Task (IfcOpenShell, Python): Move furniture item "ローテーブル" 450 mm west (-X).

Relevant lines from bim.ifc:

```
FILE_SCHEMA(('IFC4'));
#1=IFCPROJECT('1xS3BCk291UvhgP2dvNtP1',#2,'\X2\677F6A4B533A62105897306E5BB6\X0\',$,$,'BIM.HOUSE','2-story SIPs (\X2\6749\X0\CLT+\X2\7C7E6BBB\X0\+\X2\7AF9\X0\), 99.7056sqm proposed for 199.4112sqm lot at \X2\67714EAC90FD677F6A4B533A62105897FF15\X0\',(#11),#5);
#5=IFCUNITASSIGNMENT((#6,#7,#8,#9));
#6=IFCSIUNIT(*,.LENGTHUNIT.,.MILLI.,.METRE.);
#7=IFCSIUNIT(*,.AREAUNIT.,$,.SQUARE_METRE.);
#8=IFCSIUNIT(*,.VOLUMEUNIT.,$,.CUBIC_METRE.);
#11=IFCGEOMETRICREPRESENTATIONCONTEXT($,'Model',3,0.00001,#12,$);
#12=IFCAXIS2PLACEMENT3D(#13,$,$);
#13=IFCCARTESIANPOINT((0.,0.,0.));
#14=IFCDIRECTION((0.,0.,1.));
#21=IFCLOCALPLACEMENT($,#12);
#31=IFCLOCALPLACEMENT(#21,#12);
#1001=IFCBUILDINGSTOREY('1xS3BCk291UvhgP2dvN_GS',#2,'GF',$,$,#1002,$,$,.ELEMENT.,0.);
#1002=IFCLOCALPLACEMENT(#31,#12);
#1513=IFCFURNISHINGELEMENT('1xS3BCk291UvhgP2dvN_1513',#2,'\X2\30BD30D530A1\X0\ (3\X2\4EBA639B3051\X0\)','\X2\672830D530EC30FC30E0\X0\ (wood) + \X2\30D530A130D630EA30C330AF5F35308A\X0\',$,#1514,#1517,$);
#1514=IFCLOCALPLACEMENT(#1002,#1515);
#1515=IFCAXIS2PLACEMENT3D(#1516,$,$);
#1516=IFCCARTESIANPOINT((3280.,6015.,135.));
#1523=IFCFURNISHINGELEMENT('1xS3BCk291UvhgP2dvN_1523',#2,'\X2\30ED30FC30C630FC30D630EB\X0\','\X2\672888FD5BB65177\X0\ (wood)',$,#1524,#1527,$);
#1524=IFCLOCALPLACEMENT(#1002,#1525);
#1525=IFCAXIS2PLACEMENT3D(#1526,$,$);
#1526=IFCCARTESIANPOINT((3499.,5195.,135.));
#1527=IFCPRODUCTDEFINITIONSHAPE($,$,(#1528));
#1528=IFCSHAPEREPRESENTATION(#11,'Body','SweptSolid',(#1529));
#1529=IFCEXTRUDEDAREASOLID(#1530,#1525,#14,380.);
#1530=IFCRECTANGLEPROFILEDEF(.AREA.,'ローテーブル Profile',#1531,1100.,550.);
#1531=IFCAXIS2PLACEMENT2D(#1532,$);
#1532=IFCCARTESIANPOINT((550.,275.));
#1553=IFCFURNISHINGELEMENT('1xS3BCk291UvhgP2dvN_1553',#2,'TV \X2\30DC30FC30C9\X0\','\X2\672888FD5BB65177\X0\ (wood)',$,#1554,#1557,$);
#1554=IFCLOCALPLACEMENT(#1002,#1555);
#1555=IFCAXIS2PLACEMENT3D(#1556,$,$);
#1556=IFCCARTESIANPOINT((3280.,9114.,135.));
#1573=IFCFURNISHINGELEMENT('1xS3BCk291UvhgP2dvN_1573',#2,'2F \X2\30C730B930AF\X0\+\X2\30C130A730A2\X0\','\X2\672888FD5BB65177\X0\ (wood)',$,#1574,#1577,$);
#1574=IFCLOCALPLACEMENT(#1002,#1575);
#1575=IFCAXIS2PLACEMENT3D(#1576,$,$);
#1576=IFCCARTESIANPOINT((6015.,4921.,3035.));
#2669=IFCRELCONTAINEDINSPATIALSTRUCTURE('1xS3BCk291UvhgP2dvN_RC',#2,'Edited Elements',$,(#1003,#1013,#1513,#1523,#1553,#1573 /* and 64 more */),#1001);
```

```python
import ifcopenshell
import ifcopenshell.api.geometry
import ifcopenshell.util.placement
import ifcopenshell.util.unit

model = ifcopenshell.open("bim.ifc")
unit_scale = ifcopenshell.util.unit.calculate_unit_scale(model)

item = model.by_id(1523)
matrix = ifcopenshell.util.placement.get_local_placement(item.ObjectPlacement)
matrix[0, 3] -= 0.45 / unit_scale
ifcopenshell.api.geometry.edit_object_placement(model, product=item, matrix=matrix, is_si=False)

print(ifcopenshell.util.placement.get_local_placement(item.ObjectPlacement).round(3) + 0.0)

model.write("bim_updated.ifc")
```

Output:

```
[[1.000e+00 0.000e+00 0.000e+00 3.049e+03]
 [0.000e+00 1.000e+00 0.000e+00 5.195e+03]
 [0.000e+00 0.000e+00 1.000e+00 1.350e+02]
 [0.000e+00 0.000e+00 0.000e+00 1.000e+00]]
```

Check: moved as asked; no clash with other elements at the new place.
